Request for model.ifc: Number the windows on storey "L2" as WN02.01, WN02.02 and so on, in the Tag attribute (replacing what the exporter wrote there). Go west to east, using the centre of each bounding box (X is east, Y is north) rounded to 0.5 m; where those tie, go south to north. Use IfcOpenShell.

First a look at what the model holds.

```python
import ifcopenshell
import ifcopenshell.util.element
import ifcopenshell.util.placement

model = ifcopenshell.open("model.ifc")
print(model.schema)
storey = next(s for s in model.by_type("IfcBuildingStorey") if s.Name == "L2")
windows = [e for e in ifcopenshell.util.element.get_decomposition(storey) if e.is_a("IfcWindow")]
for e in sorted(windows, key=lambda e: e.id()):
    origin = ifcopenshell.util.placement.get_local_placement(e.ObjectPlacement)[:3, 3]
    print(e.id(), e.Tag, e.Name, origin.round(2) + 0.0, sep=" | ")
```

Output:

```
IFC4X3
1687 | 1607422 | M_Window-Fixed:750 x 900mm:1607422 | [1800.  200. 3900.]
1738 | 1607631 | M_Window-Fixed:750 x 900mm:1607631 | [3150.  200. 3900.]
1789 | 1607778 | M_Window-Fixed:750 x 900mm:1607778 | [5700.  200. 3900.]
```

```python
import ifcopenshell
import ifcopenshell.geom
import ifcopenshell.util.element
import ifcopenshell.util.shape

model = ifcopenshell.open("model.ifc")
settings = ifcopenshell.geom.settings()
settings.set("use-world-coords", True)


def centre(element):
    shape = ifcopenshell.geom.create_shape(settings, element)
    return ifcopenshell.util.shape.get_bbox_centroid(shape.geometry)


storey = next(s for s in model.by_type("IfcBuildingStorey") if s.Name == "L2")
windows = [e for e in ifcopenshell.util.element.get_decomposition(storey) if e.is_a("IfcWindow")]

# Insertion points can sit at a corner or the storey origin, so sort by the geometry (in metres).
centres = {e: centre(e) for e in windows}
windows.sort(key=lambda e: (round(centres[e][0] / 0.5), centres[e][1]))

for i, e in enumerate(windows, start=1):
    number = f"WN02.{i:02d}"
    e.Tag = number
    print(e.id(), number)

model.write("model_v2.ifc")
```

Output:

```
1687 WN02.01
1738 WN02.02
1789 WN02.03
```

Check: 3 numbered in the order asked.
